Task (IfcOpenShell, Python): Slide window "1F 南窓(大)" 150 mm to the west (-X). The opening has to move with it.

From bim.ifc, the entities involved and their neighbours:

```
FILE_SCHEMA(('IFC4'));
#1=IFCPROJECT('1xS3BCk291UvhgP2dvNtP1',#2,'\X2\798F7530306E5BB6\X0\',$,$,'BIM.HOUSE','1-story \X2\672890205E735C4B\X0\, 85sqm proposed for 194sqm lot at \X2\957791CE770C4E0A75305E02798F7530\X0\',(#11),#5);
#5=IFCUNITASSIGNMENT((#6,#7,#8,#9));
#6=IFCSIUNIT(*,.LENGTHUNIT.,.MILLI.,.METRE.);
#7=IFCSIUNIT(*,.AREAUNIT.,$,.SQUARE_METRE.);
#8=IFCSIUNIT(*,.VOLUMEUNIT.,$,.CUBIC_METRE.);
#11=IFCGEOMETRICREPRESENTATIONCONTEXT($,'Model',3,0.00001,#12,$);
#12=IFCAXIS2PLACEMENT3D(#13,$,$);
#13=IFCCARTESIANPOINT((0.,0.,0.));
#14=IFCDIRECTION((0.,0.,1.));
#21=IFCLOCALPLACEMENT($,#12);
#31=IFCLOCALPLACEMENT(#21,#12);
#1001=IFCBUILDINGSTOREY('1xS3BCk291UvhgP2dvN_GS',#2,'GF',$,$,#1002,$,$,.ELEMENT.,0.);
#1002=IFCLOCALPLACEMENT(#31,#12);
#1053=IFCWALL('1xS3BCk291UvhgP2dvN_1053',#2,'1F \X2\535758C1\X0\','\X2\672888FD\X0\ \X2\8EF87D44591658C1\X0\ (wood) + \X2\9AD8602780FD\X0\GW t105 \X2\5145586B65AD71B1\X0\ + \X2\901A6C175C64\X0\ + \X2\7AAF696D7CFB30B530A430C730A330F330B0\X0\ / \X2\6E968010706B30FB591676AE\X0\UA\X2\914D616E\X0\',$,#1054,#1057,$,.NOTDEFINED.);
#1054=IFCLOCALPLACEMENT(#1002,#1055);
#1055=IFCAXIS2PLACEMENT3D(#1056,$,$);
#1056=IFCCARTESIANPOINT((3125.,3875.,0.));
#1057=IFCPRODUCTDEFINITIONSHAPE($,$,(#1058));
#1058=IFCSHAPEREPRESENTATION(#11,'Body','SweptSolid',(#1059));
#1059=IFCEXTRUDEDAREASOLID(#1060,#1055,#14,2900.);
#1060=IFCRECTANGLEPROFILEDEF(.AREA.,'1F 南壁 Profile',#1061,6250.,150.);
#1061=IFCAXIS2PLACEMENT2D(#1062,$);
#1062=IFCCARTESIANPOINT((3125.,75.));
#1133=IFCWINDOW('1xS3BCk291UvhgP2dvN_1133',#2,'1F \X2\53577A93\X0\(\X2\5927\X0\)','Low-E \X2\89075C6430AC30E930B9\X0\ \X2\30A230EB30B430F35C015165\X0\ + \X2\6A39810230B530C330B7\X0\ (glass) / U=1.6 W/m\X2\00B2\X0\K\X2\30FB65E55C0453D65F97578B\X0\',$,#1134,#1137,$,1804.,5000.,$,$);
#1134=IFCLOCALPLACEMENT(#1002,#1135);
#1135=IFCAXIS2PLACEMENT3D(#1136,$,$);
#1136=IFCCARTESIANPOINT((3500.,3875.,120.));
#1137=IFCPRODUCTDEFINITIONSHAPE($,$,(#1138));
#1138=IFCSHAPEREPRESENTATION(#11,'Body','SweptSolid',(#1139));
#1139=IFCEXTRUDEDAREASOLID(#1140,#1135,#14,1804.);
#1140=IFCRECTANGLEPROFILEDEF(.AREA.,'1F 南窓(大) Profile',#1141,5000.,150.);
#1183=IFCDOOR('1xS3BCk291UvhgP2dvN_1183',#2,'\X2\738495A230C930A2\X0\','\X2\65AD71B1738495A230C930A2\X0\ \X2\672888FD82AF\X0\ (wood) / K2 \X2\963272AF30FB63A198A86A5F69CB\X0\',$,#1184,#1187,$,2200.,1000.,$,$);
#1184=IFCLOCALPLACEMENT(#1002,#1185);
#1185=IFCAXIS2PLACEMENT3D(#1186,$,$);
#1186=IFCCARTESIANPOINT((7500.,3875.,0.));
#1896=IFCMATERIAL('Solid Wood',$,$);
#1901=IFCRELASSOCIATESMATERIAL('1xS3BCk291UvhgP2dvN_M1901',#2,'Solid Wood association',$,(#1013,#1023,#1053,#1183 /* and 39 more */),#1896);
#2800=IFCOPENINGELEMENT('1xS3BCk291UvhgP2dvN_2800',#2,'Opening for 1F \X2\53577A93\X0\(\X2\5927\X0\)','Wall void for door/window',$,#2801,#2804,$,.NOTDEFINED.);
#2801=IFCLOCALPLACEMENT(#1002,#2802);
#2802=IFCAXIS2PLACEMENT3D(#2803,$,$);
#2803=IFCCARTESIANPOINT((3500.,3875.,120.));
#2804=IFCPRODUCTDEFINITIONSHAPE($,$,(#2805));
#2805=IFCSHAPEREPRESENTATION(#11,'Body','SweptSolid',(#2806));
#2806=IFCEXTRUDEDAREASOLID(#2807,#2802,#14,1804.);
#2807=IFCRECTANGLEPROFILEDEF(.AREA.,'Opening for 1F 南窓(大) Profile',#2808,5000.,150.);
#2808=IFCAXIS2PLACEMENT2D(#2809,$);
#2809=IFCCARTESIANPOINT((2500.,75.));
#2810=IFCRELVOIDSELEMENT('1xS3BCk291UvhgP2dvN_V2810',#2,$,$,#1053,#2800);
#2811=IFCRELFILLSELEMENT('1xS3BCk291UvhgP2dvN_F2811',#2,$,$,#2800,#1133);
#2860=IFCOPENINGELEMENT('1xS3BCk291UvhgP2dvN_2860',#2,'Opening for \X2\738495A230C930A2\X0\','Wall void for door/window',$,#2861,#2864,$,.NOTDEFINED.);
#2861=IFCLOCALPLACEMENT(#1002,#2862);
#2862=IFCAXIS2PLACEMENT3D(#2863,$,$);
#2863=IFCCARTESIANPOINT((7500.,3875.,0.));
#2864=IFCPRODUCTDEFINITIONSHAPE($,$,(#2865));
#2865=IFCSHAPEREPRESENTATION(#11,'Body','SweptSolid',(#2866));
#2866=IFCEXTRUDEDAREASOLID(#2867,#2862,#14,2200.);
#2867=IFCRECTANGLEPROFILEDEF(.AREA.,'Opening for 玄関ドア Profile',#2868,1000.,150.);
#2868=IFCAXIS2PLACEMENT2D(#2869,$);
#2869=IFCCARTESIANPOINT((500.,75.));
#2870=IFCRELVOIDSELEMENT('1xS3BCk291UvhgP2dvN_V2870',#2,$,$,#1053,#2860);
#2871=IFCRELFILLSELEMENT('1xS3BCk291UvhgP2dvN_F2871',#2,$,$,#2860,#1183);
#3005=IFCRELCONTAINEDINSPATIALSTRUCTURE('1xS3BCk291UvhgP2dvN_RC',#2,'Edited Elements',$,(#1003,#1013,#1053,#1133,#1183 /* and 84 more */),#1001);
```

```python
import ifcopenshell
import ifcopenshell.api.geometry
import ifcopenshell.util.placement
import ifcopenshell.util.unit

model = ifcopenshell.open("bim.ifc")
unit_scale = ifcopenshell.util.unit.calculate_unit_scale(model)

window = model.by_guid("1xS3BCk291UvhgP2dvN_1133")
opening = window.FillsVoids[0].RelatingOpeningElement
wall = opening.VoidsElements[0].RelatingBuildingElement

wall_matrix = ifcopenshell.util.placement.get_local_placement(wall.ObjectPlacement)
shift = wall_matrix[:3, 0] * -0.15 / unit_scale
before = ifcopenshell.util.placement.get_local_placement(window.ObjectPlacement)[:3, 3].copy()

# The window is not placed relative to its opening, so move both.
for product in (opening, window):
    matrix = ifcopenshell.util.placement.get_local_placement(product.ObjectPlacement)
    matrix[:3, 3] += shift
    ifcopenshell.api.geometry.edit_object_placement(model, product=product, matrix=matrix, is_si=False)

after = ifcopenshell.util.placement.get_local_placement(window.ObjectPlacement)[:3, 3]
print("window moved by", (after - before).round(3) + 0.0)

model.write("bim_rev.ifc")
```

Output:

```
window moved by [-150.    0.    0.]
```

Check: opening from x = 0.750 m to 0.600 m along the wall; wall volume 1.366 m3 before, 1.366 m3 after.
